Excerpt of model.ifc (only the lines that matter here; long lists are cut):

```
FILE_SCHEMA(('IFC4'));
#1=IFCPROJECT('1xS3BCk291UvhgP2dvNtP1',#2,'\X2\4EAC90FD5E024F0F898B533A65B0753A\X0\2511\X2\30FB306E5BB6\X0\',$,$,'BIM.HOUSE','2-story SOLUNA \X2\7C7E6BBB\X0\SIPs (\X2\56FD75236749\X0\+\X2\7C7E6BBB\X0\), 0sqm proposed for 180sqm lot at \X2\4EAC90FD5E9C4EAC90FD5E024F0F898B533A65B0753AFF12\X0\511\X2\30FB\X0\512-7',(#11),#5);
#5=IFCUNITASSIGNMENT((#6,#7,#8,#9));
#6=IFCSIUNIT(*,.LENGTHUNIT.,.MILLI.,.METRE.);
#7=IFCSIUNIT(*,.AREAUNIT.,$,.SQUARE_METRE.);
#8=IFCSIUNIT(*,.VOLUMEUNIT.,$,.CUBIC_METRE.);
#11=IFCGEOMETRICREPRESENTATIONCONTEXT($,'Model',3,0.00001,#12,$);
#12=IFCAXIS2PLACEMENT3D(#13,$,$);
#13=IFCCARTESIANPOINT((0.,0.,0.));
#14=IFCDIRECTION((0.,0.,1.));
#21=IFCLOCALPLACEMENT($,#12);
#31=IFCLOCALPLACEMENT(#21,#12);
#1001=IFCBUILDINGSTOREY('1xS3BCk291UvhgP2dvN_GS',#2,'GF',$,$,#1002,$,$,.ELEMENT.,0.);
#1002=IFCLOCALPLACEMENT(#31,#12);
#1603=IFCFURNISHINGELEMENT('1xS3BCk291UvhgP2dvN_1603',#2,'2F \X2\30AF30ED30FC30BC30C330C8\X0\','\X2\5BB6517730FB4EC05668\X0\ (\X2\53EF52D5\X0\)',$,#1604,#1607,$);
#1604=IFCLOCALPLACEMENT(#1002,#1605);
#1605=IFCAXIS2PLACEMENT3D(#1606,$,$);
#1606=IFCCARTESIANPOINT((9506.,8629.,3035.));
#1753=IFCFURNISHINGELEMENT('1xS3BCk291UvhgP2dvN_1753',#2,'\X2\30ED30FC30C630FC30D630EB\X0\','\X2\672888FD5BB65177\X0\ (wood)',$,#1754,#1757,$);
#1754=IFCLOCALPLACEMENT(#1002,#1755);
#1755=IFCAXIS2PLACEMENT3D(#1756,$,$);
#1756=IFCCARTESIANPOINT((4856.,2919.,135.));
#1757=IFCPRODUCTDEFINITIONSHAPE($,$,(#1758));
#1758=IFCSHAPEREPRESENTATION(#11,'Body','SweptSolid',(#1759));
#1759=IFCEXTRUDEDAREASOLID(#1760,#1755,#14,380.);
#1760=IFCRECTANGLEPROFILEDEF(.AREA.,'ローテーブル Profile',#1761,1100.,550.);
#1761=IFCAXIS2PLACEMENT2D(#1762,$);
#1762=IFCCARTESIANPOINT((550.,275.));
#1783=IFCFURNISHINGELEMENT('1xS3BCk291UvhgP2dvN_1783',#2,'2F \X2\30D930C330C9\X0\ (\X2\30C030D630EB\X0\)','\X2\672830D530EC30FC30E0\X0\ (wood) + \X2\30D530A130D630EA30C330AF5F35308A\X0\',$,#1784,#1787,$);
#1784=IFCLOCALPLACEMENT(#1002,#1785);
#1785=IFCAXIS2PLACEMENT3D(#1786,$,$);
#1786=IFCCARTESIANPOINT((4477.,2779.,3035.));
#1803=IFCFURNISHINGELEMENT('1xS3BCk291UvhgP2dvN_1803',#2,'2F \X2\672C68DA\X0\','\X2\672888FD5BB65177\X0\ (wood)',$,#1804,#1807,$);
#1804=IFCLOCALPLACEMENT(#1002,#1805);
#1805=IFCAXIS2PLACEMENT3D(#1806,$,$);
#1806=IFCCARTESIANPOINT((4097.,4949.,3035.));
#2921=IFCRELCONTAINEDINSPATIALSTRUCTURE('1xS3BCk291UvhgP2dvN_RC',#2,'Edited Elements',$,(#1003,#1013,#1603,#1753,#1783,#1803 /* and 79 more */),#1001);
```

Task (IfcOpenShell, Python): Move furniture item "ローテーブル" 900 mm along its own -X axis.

```python
import ifcopenshell
import ifcopenshell.api.geometry
import ifcopenshell.util.placement
import ifcopenshell.util.unit

model = ifcopenshell.open("model.ifc")
unit_scale = ifcopenshell.util.unit.calculate_unit_scale(model)

item = model.by_id(1753)
matrix = ifcopenshell.util.placement.get_local_placement(item.ObjectPlacement)
matrix[:3, 3] -= matrix[:3, 0] * 0.9 / unit_scale
ifcopenshell.api.geometry.edit_object_placement(model, product=item, matrix=matrix, is_si=False)

print(ifcopenshell.util.placement.get_local_placement(item.ObjectPlacement).round(3) + 0.0)

model.write("model_edited.ifc")
```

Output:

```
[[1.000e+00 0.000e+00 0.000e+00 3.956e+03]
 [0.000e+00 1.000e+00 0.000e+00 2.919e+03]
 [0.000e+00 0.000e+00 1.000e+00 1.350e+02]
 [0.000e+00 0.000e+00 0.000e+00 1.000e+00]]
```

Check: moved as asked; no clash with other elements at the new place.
